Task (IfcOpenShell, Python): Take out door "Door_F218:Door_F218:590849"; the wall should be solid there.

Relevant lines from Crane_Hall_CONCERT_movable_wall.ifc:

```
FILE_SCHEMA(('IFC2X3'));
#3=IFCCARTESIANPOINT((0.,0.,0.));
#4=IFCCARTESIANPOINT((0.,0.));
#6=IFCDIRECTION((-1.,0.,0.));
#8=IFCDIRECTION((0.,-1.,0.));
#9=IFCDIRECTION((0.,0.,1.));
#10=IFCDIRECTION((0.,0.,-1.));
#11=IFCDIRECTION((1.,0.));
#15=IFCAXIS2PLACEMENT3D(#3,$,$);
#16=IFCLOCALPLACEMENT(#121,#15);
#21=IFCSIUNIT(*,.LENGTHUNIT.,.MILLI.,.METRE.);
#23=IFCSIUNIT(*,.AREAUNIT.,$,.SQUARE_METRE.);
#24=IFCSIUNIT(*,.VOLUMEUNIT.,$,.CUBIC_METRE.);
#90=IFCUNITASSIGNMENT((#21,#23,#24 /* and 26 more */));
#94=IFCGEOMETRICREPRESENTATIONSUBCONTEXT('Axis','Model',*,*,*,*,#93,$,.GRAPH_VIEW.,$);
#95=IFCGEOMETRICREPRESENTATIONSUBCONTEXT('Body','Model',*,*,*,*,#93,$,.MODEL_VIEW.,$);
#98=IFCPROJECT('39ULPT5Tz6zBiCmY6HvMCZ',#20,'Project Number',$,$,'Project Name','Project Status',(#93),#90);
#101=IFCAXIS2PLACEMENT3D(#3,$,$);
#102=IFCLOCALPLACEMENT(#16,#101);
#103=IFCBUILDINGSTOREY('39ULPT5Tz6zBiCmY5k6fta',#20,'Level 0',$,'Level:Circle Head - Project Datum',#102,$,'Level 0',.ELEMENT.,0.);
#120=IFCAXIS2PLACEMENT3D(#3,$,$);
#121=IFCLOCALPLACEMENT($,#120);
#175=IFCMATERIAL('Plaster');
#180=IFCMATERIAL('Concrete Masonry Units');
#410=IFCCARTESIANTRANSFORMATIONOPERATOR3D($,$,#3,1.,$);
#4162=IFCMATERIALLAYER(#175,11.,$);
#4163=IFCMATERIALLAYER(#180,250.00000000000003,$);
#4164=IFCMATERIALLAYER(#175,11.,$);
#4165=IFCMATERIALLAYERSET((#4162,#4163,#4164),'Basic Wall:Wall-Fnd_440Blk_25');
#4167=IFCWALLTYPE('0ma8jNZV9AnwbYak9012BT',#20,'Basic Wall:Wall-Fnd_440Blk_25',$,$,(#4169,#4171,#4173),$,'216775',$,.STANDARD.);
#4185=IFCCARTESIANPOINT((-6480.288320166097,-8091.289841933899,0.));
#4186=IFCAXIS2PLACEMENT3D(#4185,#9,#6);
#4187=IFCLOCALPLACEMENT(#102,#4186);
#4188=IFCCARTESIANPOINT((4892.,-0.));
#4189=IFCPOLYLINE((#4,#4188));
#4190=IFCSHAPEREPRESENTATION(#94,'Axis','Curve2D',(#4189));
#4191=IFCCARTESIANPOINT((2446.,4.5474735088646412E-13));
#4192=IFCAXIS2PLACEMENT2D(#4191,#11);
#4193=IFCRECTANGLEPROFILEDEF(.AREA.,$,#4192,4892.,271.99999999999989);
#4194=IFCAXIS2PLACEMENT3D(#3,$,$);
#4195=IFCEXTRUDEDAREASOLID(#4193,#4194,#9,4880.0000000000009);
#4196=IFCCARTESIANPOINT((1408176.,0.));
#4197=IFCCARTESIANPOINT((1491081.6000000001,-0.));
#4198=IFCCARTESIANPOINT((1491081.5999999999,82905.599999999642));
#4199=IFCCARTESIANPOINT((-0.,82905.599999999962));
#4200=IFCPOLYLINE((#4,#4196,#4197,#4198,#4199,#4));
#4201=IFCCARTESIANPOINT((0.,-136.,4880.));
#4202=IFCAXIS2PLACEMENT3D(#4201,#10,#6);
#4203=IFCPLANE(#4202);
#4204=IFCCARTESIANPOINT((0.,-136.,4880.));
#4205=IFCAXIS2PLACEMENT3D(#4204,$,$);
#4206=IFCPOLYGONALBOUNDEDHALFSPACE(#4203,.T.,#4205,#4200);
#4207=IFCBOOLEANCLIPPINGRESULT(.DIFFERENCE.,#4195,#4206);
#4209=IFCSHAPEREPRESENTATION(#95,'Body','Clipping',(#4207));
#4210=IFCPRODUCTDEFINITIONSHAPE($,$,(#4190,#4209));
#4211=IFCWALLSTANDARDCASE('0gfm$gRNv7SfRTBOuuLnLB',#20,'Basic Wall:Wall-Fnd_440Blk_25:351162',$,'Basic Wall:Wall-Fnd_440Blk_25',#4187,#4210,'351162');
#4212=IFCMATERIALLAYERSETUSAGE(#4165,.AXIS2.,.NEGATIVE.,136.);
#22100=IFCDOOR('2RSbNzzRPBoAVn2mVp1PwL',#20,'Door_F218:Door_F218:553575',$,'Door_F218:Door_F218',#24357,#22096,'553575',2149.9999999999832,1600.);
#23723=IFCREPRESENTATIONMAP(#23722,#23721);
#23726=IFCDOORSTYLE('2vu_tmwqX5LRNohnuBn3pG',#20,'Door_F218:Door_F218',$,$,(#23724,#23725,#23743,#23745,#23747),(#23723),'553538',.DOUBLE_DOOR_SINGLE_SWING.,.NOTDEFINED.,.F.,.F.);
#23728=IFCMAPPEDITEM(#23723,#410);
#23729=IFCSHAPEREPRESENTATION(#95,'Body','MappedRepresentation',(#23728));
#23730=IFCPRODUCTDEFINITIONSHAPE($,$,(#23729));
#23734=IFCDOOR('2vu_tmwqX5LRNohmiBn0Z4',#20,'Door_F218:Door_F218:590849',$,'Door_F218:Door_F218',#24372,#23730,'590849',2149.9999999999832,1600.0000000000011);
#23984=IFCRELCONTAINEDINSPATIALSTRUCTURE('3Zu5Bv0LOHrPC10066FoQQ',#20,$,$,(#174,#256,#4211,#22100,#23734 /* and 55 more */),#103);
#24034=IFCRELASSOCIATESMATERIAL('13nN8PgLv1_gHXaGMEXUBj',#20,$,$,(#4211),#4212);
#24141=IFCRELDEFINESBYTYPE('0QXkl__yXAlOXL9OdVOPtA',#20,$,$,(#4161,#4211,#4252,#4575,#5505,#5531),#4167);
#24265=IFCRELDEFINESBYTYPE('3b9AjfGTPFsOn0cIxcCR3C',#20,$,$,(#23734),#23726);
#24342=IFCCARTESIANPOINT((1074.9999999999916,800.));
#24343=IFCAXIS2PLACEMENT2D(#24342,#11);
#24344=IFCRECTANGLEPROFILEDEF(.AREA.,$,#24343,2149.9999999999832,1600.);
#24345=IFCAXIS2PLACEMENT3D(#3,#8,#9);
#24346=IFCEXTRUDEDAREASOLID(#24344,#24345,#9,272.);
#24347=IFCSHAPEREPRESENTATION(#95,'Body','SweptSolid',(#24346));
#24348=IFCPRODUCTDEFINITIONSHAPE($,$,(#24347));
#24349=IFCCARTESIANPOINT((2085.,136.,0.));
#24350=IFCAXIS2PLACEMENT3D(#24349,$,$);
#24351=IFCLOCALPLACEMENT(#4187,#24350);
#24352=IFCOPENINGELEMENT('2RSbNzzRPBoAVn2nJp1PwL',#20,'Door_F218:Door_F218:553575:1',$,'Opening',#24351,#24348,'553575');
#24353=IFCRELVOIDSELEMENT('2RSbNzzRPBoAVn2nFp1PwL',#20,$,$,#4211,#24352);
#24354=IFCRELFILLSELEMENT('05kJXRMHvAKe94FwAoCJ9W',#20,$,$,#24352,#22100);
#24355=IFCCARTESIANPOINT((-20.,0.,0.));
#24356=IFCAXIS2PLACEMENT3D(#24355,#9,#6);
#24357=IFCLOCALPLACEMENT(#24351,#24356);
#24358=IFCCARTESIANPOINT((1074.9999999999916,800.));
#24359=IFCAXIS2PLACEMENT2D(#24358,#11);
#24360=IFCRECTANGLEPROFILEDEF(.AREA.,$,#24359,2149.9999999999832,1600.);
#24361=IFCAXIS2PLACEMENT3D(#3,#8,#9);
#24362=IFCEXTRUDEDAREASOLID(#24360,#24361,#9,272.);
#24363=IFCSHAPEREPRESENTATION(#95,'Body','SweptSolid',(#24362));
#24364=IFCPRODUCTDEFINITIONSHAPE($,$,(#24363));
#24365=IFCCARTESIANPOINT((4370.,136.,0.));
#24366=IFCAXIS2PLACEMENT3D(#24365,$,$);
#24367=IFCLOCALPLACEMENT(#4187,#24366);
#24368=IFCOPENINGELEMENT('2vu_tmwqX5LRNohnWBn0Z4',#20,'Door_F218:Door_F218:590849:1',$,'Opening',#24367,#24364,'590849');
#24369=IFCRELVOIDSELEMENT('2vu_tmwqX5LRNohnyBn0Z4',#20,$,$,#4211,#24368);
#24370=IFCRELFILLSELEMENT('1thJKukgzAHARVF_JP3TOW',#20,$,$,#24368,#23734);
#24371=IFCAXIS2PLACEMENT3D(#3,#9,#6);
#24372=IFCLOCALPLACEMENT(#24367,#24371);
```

```python
import ifcopenshell
import ifcopenshell.api.feature
import ifcopenshell.api.root
import ifcopenshell.geom
import ifcopenshell.util.shape

model = ifcopenshell.open("Crane_Hall_CONCERT_movable_wall.ifc")
settings = ifcopenshell.geom.settings()


def volume(element):
    """Net volume in cubic metres, openings subtracted."""
    shape = ifcopenshell.geom.create_shape(settings, element)
    return ifcopenshell.util.shape.get_volume(shape.geometry)


door = model.by_guid("2vu_tmwqX5LRNohmiBn0Z4")
opening = door.FillsVoids[0].RelatingOpeningElement
wall = opening.VoidsElements[0].RelatingBuildingElement
before = volume(wall)

ifcopenshell.api.root.remove_product(model, product=door)
ifcopenshell.api.feature.remove_feature(model, feature=opening)

after = volume(wall)

print(f"wall volume {before:.3f} -> {after:.3f} m3")

model.write("Crane_Hall_CONCERT_movable_wall_updated.ifc")
```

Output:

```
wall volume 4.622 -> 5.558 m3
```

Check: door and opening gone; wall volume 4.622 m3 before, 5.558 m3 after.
